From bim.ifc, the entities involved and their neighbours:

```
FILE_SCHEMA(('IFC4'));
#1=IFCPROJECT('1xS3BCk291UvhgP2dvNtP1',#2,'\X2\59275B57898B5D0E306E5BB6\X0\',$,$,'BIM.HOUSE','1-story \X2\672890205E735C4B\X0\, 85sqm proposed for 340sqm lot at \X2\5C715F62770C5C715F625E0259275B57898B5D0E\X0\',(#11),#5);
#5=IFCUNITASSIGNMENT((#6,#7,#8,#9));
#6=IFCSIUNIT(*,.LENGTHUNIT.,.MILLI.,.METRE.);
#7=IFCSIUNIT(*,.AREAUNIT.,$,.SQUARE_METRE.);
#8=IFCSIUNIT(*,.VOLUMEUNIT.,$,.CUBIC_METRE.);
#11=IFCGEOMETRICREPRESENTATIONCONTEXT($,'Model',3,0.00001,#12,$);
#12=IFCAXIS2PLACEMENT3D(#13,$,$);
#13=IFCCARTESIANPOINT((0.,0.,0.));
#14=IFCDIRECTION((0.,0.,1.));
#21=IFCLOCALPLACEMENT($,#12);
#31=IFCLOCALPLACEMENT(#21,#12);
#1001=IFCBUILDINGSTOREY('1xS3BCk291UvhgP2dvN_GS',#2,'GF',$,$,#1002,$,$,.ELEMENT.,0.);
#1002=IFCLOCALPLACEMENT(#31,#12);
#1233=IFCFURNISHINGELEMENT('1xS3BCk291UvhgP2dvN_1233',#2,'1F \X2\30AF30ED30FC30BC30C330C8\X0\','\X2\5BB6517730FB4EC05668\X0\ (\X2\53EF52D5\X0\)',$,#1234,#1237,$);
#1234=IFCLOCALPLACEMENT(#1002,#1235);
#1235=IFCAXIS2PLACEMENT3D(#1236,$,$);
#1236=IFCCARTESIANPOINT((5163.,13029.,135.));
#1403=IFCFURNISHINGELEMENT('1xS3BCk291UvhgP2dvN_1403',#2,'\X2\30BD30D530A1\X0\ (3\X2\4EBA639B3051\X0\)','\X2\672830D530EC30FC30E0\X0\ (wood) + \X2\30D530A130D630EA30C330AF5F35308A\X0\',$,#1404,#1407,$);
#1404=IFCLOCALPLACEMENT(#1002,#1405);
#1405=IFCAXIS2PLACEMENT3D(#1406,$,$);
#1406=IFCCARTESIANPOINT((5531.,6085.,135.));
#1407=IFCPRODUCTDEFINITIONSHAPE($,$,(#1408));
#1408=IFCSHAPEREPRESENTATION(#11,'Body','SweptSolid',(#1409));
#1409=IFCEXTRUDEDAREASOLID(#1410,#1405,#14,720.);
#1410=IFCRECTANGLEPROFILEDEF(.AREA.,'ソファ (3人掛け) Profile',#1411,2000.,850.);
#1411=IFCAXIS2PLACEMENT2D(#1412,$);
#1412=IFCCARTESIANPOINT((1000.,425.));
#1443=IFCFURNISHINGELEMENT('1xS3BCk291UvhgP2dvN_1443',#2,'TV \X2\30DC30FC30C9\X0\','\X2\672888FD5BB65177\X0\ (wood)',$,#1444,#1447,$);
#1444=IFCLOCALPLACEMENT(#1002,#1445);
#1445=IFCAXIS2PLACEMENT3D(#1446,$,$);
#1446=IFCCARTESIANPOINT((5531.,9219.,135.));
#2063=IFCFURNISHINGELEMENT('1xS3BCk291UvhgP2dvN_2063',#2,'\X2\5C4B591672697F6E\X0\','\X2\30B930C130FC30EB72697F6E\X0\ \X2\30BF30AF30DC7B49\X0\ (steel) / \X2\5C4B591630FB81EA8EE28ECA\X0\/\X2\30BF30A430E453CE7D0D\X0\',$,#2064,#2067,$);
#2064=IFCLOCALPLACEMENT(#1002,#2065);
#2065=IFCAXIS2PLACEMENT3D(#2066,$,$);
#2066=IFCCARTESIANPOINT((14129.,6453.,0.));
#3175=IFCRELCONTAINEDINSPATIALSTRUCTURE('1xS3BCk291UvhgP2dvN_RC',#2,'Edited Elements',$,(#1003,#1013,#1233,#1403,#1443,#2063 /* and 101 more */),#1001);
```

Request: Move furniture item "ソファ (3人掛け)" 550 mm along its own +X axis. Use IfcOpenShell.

```python
import ifcopenshell
import ifcopenshell.api.geometry
import ifcopenshell.util.placement
import ifcopenshell.util.unit

model = ifcopenshell.open("bim.ifc")
unit_scale = ifcopenshell.util.unit.calculate_unit_scale(model)

item = model.by_guid("1xS3BCk291UvhgP2dvN_1403")
matrix = ifcopenshell.util.placement.get_local_placement(item.ObjectPlacement)
matrix[:3, 3] += matrix[:3, 0] * 0.55 / unit_scale
ifcopenshell.api.geometry.edit_object_placement(model, product=item, matrix=matrix, is_si=False)

print(ifcopenshell.util.placement.get_local_placement(item.ObjectPlacement).round(3) + 0.0)

model.write("bim_rev.ifc")
```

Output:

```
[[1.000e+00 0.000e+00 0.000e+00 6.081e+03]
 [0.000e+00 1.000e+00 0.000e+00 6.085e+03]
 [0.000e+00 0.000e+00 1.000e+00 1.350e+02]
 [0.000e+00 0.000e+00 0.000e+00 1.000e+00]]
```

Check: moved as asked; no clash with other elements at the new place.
